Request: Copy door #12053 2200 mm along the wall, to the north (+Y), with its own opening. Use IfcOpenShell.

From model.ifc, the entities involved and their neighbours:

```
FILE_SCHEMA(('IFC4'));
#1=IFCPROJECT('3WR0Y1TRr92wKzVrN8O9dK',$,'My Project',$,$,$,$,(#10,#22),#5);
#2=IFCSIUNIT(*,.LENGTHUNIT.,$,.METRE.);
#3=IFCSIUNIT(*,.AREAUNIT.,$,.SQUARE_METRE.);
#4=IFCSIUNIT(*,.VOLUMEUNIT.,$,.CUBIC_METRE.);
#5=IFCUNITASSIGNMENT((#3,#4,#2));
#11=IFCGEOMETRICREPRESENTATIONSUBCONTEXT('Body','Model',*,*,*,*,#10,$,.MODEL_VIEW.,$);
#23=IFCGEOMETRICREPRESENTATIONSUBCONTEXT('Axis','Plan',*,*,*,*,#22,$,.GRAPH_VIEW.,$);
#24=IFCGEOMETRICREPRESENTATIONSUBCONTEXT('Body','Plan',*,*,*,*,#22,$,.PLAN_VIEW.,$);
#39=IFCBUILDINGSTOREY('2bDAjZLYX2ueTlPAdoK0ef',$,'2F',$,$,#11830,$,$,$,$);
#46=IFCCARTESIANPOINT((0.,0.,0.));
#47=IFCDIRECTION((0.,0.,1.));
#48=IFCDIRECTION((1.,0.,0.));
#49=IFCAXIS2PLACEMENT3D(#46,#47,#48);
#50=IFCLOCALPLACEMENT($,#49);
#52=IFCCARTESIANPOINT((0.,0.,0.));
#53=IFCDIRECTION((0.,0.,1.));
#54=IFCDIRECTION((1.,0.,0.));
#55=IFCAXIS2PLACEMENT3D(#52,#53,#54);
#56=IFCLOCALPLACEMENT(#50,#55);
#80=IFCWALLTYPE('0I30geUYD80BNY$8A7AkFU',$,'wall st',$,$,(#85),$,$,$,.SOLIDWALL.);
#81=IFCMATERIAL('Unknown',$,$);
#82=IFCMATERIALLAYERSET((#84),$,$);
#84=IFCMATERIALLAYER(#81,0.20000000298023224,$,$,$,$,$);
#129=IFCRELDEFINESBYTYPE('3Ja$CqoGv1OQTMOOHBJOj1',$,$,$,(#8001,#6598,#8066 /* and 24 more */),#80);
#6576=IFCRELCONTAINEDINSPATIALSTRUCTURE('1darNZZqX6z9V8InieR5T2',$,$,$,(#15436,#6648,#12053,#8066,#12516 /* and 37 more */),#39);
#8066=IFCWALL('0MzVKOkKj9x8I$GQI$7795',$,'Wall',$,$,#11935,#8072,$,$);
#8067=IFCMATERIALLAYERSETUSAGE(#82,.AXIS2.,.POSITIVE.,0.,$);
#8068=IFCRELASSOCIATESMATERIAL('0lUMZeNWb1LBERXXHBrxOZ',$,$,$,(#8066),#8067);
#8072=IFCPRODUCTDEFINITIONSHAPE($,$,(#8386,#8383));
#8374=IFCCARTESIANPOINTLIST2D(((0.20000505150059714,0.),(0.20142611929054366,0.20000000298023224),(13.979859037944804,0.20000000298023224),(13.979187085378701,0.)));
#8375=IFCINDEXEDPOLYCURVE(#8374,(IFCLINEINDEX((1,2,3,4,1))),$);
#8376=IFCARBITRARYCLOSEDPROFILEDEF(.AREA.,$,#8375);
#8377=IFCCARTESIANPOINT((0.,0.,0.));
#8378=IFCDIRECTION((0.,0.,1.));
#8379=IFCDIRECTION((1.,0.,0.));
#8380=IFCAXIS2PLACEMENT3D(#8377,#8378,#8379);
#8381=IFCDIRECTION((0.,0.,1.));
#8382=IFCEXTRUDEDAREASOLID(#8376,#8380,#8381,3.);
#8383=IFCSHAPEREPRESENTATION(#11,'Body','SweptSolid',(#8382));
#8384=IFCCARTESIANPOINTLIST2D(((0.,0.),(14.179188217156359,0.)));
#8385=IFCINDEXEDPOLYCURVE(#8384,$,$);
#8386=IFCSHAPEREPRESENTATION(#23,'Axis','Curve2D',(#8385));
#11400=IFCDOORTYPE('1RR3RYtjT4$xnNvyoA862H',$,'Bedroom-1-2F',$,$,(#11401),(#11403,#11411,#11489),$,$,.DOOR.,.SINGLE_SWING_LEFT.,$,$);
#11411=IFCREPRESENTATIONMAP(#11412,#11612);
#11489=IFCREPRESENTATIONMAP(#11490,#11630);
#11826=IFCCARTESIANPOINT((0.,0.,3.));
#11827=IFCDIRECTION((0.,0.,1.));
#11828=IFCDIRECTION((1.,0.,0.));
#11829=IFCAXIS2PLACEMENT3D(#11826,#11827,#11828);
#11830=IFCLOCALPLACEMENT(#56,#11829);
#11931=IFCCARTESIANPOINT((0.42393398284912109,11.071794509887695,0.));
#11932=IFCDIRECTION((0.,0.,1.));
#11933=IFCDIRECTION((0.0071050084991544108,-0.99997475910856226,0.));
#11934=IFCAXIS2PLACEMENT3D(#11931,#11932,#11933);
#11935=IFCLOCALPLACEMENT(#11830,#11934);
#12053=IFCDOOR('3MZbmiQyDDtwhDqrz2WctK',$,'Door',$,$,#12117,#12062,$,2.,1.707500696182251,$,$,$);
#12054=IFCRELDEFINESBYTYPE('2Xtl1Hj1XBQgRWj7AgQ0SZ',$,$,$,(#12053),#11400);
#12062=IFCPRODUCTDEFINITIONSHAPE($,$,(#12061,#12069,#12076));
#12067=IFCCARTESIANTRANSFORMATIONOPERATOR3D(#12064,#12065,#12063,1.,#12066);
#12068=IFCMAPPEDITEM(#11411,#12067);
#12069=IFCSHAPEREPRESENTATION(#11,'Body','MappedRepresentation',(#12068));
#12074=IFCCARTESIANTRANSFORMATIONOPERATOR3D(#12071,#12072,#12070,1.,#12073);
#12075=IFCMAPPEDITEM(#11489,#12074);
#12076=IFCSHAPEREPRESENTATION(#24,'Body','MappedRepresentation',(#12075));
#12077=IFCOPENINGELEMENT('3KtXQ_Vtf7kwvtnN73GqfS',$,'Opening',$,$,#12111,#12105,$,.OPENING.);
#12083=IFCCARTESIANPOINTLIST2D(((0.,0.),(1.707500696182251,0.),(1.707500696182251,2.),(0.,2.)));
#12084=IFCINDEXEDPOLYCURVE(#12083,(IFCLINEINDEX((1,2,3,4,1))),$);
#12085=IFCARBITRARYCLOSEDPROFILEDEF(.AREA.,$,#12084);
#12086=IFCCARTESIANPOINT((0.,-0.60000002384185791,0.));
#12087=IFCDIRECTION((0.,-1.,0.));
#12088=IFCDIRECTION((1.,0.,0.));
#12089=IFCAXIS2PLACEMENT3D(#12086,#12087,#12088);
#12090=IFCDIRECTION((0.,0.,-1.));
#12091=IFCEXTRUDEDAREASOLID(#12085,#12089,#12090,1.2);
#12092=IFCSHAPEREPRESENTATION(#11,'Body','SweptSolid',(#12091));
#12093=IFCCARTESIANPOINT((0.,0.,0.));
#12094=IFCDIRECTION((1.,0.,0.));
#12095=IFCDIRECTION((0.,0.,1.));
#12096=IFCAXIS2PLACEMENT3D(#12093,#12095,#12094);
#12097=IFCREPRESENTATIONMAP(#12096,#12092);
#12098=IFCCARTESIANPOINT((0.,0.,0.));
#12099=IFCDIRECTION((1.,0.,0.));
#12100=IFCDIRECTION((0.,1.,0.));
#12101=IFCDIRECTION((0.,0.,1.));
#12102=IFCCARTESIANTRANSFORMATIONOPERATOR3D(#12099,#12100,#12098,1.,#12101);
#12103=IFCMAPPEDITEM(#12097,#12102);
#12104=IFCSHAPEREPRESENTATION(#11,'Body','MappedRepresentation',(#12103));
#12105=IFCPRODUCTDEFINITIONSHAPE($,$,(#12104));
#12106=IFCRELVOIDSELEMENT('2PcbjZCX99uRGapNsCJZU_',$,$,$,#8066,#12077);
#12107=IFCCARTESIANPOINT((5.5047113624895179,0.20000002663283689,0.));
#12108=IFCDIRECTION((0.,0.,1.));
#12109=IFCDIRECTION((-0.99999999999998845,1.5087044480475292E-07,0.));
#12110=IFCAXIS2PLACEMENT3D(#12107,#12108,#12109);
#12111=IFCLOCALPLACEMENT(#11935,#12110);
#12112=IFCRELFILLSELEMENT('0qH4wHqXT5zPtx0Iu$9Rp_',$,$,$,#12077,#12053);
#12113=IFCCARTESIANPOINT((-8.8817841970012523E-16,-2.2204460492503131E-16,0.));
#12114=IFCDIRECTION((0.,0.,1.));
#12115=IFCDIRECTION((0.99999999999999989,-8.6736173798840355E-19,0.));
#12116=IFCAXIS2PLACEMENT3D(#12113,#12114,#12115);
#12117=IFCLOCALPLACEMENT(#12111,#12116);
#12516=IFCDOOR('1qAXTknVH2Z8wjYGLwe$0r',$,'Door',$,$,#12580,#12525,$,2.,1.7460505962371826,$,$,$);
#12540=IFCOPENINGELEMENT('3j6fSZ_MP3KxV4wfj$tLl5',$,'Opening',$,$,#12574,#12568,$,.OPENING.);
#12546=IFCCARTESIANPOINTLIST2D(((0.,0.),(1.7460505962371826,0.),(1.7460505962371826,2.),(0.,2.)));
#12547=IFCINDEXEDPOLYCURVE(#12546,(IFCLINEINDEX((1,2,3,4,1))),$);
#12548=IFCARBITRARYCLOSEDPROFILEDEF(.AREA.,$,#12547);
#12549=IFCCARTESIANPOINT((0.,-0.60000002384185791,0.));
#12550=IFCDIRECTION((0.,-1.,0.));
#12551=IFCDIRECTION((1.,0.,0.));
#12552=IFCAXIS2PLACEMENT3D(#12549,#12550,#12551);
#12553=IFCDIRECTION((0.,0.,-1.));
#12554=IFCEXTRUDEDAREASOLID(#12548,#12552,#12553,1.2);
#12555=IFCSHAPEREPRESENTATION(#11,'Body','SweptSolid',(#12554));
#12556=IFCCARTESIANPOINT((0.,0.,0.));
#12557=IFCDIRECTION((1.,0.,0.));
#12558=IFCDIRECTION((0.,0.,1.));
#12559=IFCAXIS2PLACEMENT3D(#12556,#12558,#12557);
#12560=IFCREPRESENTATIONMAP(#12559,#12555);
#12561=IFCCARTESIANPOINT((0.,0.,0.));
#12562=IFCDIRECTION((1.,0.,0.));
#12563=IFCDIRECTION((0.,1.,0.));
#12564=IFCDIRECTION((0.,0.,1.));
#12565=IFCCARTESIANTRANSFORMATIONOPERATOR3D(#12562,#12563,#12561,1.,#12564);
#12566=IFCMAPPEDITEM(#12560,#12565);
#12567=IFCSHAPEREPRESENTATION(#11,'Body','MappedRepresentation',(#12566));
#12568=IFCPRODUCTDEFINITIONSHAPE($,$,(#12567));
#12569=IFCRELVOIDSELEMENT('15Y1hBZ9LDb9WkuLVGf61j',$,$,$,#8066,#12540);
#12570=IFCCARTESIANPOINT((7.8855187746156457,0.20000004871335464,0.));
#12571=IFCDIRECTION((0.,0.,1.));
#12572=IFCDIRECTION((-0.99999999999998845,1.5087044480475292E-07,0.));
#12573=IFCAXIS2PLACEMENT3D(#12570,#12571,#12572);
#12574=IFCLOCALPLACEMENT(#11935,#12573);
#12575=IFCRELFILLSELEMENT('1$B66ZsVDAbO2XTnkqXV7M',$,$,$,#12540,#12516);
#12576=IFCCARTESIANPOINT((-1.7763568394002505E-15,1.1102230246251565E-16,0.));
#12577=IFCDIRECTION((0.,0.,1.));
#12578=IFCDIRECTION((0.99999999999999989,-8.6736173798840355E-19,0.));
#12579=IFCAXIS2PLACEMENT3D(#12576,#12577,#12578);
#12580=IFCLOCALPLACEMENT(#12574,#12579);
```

```python
import ifcopenshell
import ifcopenshell.api.feature
import ifcopenshell.api.geometry
import ifcopenshell.api.root
import ifcopenshell.geom
import ifcopenshell.util.element
import ifcopenshell.util.placement
import ifcopenshell.util.shape
import ifcopenshell.util.unit

model = ifcopenshell.open("model.ifc")
unit_scale = ifcopenshell.util.unit.calculate_unit_scale(model)
settings = ifcopenshell.geom.settings()


def volume(element):
    """Net volume in cubic metres, openings subtracted."""
    shape = ifcopenshell.geom.create_shape(settings, element)
    return ifcopenshell.util.shape.get_volume(shape.geometry)


door = model.by_guid("3MZbmiQyDDtwhDqrz2WctK")
opening = door.FillsVoids[0].RelatingOpeningElement
wall = opening.VoidsElements[0].RelatingBuildingElement
before = volume(wall)
shift = ifcopenshell.util.placement.get_local_placement(wall.ObjectPlacement)[:3, 0] * -2.2 / unit_scale

# copy_class copies the void relationship, type, container and properties, but no geometry.
new_opening = ifcopenshell.api.root.copy_class(model, product=opening)
new_opening.Representation = ifcopenshell.util.element.copy_deep(
    model, opening.Representation, exclude=["IfcGeometricRepresentationContext", "IfcRepresentationMap"]
)
new_door = ifcopenshell.api.root.copy_class(model, product=door)
new_door.Representation = ifcopenshell.util.element.copy_deep(
    model, door.Representation, exclude=["IfcGeometricRepresentationContext", "IfcRepresentationMap"]
)
ifcopenshell.api.feature.add_filling(model, opening=new_opening, element=new_door)

for old, new in ((opening, new_opening), (door, new_door)):
    matrix = ifcopenshell.util.placement.get_local_placement(old.ObjectPlacement)
    matrix[:3, 3] += shift
    ifcopenshell.api.geometry.edit_object_placement(model, product=new, matrix=matrix, is_si=False)

after = volume(wall)

print(f"wall volume {before:.3f} -> {after:.3f} m3")

model.write("model_v2.ifc")
```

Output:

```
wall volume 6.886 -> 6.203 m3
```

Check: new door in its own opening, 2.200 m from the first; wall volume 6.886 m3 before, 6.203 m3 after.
